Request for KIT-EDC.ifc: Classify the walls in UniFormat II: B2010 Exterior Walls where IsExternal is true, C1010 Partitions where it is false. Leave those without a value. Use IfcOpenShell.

First a look at what the model holds.

```python
import ifcopenshell
import ifcopenshell.util.element

model = ifcopenshell.open("KIT-EDC.ifc")
print(model.schema)
print("classifications:", [c.Name for c in model.by_type("IfcClassification")])
values = [ifcopenshell.util.element.get_pset(e, "Pset_WallCommon", "IsExternal") for e in model.by_type("IfcWall")]
for value in (True, False, None):
    print("IsExternal", value, values.count(value))
```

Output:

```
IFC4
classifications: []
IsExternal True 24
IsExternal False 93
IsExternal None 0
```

```python
import ifcopenshell
import ifcopenshell.api.classification
import ifcopenshell.util.element

model = ifcopenshell.open("KIT-EDC.ifc")

system = ifcopenshell.api.classification.add_classification(model, classification="UniFormat II")

walls = model.by_type("IfcWall")
external = {e: ifcopenshell.util.element.get_pset(e, "Pset_WallCommon", "IsExternal") for e in walls}
for flag, code, name in ((True, "B2010", "Exterior Walls"), (False, "C1010", "Partitions")):
    products = [e for e in walls if external[e] is flag]
    ifcopenshell.api.classification.add_reference(
        model, products=products, classification=system, identification=code, name=name
    )
    print(code, len(products))

model.write("KIT-EDC_edited.ifc")
```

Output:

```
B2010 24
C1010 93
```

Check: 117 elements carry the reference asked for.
